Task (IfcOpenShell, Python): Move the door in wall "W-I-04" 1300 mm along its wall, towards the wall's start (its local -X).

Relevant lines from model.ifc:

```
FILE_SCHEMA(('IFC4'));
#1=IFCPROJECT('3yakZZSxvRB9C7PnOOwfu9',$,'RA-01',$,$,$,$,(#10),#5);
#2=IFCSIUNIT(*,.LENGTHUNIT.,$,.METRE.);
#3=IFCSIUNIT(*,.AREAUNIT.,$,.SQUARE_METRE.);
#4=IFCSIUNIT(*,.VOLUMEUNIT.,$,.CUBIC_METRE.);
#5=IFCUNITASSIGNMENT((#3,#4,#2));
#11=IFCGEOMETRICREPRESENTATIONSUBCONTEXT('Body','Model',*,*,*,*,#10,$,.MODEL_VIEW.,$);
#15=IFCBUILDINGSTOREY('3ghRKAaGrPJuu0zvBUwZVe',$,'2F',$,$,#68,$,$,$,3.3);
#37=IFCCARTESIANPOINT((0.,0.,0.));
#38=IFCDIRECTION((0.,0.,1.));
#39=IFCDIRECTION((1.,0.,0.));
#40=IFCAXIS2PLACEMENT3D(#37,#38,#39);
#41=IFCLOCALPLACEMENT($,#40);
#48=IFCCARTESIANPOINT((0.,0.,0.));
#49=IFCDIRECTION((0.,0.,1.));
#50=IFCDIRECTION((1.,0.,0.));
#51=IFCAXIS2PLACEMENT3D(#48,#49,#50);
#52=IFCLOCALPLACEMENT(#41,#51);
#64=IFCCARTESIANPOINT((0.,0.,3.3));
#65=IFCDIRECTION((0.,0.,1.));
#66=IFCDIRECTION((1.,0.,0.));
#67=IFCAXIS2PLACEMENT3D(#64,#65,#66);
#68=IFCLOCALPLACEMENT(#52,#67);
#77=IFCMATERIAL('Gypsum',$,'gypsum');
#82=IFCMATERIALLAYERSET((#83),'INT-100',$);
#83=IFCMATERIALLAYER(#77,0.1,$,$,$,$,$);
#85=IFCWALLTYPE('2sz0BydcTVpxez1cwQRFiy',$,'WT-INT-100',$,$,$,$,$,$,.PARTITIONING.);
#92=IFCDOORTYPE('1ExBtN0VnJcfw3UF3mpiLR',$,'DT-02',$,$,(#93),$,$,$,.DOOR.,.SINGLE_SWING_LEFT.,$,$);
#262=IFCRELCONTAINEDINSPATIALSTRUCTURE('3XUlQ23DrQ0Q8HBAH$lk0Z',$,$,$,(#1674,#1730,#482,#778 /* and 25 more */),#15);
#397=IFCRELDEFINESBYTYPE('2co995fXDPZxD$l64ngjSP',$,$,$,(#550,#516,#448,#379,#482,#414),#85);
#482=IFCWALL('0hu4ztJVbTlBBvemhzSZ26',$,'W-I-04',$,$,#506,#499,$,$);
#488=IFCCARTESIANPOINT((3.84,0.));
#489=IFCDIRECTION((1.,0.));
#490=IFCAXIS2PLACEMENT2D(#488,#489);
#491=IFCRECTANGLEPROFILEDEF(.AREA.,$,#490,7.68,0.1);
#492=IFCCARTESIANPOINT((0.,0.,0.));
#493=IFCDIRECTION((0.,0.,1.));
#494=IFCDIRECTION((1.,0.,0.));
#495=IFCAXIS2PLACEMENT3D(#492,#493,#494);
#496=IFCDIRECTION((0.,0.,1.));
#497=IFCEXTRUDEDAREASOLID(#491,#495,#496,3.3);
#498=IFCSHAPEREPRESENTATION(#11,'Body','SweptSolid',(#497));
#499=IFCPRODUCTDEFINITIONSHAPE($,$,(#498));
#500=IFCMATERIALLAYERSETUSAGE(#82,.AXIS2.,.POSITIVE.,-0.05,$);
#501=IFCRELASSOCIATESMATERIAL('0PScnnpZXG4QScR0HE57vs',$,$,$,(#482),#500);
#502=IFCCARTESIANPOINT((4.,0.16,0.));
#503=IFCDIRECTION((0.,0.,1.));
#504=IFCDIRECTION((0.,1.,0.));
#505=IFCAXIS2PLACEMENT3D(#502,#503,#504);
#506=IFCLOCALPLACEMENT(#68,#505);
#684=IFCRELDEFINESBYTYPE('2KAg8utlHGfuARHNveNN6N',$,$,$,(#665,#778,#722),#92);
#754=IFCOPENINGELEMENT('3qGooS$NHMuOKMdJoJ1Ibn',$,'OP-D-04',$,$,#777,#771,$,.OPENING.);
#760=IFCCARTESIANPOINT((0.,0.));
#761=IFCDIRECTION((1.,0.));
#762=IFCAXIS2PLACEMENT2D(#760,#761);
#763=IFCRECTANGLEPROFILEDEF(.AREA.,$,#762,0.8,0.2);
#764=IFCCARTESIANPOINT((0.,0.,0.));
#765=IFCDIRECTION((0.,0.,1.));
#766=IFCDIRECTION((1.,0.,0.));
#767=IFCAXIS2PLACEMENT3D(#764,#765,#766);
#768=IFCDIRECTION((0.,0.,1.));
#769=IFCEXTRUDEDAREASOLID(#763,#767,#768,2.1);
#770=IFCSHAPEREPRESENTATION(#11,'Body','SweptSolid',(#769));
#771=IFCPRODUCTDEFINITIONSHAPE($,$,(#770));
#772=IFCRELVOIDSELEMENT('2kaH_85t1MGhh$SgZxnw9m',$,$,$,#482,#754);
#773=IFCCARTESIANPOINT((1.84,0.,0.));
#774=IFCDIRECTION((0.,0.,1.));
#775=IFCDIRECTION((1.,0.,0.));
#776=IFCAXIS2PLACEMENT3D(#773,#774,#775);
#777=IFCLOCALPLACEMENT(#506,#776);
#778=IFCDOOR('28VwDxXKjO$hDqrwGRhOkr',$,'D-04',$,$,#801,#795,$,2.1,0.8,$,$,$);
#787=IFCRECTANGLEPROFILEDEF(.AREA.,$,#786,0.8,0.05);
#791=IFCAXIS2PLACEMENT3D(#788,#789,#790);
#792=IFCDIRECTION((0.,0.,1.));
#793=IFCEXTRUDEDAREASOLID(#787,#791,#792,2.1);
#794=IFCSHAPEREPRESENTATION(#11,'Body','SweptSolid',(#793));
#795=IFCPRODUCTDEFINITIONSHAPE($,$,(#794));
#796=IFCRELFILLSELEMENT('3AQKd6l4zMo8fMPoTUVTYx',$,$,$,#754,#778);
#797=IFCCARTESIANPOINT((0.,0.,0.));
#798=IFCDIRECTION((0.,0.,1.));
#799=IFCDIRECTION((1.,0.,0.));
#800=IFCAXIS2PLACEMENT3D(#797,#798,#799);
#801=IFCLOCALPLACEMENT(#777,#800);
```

```python
import ifcopenshell
import ifcopenshell.api.geometry
import ifcopenshell.util.placement

model = ifcopenshell.open("model.ifc")

door = model.by_guid("28VwDxXKjO$hDqrwGRhOkr")
opening = door.FillsVoids[0].RelatingOpeningElement
wall = opening.VoidsElements[0].RelatingBuildingElement

wall_matrix = ifcopenshell.util.placement.get_local_placement(wall.ObjectPlacement)
shift = wall_matrix[:3, 0] * -1.3
before = ifcopenshell.util.placement.get_local_placement(door.ObjectPlacement)[:3, 3].copy()

# The door is placed relative to its opening, so it follows when the opening moves.
matrix = ifcopenshell.util.placement.get_local_placement(opening.ObjectPlacement)
matrix[:3, 3] += shift
ifcopenshell.api.geometry.edit_object_placement(
    model, product=opening, matrix=matrix, is_si=False, should_transform_children=True
)

after = ifcopenshell.util.placement.get_local_placement(door.ObjectPlacement)[:3, 3]
print("door moved by", (after - before).round(3) + 0.0)

model.write("model_rev.ifc")
```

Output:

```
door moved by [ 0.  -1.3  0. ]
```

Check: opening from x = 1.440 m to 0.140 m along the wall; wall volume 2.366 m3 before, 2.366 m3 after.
